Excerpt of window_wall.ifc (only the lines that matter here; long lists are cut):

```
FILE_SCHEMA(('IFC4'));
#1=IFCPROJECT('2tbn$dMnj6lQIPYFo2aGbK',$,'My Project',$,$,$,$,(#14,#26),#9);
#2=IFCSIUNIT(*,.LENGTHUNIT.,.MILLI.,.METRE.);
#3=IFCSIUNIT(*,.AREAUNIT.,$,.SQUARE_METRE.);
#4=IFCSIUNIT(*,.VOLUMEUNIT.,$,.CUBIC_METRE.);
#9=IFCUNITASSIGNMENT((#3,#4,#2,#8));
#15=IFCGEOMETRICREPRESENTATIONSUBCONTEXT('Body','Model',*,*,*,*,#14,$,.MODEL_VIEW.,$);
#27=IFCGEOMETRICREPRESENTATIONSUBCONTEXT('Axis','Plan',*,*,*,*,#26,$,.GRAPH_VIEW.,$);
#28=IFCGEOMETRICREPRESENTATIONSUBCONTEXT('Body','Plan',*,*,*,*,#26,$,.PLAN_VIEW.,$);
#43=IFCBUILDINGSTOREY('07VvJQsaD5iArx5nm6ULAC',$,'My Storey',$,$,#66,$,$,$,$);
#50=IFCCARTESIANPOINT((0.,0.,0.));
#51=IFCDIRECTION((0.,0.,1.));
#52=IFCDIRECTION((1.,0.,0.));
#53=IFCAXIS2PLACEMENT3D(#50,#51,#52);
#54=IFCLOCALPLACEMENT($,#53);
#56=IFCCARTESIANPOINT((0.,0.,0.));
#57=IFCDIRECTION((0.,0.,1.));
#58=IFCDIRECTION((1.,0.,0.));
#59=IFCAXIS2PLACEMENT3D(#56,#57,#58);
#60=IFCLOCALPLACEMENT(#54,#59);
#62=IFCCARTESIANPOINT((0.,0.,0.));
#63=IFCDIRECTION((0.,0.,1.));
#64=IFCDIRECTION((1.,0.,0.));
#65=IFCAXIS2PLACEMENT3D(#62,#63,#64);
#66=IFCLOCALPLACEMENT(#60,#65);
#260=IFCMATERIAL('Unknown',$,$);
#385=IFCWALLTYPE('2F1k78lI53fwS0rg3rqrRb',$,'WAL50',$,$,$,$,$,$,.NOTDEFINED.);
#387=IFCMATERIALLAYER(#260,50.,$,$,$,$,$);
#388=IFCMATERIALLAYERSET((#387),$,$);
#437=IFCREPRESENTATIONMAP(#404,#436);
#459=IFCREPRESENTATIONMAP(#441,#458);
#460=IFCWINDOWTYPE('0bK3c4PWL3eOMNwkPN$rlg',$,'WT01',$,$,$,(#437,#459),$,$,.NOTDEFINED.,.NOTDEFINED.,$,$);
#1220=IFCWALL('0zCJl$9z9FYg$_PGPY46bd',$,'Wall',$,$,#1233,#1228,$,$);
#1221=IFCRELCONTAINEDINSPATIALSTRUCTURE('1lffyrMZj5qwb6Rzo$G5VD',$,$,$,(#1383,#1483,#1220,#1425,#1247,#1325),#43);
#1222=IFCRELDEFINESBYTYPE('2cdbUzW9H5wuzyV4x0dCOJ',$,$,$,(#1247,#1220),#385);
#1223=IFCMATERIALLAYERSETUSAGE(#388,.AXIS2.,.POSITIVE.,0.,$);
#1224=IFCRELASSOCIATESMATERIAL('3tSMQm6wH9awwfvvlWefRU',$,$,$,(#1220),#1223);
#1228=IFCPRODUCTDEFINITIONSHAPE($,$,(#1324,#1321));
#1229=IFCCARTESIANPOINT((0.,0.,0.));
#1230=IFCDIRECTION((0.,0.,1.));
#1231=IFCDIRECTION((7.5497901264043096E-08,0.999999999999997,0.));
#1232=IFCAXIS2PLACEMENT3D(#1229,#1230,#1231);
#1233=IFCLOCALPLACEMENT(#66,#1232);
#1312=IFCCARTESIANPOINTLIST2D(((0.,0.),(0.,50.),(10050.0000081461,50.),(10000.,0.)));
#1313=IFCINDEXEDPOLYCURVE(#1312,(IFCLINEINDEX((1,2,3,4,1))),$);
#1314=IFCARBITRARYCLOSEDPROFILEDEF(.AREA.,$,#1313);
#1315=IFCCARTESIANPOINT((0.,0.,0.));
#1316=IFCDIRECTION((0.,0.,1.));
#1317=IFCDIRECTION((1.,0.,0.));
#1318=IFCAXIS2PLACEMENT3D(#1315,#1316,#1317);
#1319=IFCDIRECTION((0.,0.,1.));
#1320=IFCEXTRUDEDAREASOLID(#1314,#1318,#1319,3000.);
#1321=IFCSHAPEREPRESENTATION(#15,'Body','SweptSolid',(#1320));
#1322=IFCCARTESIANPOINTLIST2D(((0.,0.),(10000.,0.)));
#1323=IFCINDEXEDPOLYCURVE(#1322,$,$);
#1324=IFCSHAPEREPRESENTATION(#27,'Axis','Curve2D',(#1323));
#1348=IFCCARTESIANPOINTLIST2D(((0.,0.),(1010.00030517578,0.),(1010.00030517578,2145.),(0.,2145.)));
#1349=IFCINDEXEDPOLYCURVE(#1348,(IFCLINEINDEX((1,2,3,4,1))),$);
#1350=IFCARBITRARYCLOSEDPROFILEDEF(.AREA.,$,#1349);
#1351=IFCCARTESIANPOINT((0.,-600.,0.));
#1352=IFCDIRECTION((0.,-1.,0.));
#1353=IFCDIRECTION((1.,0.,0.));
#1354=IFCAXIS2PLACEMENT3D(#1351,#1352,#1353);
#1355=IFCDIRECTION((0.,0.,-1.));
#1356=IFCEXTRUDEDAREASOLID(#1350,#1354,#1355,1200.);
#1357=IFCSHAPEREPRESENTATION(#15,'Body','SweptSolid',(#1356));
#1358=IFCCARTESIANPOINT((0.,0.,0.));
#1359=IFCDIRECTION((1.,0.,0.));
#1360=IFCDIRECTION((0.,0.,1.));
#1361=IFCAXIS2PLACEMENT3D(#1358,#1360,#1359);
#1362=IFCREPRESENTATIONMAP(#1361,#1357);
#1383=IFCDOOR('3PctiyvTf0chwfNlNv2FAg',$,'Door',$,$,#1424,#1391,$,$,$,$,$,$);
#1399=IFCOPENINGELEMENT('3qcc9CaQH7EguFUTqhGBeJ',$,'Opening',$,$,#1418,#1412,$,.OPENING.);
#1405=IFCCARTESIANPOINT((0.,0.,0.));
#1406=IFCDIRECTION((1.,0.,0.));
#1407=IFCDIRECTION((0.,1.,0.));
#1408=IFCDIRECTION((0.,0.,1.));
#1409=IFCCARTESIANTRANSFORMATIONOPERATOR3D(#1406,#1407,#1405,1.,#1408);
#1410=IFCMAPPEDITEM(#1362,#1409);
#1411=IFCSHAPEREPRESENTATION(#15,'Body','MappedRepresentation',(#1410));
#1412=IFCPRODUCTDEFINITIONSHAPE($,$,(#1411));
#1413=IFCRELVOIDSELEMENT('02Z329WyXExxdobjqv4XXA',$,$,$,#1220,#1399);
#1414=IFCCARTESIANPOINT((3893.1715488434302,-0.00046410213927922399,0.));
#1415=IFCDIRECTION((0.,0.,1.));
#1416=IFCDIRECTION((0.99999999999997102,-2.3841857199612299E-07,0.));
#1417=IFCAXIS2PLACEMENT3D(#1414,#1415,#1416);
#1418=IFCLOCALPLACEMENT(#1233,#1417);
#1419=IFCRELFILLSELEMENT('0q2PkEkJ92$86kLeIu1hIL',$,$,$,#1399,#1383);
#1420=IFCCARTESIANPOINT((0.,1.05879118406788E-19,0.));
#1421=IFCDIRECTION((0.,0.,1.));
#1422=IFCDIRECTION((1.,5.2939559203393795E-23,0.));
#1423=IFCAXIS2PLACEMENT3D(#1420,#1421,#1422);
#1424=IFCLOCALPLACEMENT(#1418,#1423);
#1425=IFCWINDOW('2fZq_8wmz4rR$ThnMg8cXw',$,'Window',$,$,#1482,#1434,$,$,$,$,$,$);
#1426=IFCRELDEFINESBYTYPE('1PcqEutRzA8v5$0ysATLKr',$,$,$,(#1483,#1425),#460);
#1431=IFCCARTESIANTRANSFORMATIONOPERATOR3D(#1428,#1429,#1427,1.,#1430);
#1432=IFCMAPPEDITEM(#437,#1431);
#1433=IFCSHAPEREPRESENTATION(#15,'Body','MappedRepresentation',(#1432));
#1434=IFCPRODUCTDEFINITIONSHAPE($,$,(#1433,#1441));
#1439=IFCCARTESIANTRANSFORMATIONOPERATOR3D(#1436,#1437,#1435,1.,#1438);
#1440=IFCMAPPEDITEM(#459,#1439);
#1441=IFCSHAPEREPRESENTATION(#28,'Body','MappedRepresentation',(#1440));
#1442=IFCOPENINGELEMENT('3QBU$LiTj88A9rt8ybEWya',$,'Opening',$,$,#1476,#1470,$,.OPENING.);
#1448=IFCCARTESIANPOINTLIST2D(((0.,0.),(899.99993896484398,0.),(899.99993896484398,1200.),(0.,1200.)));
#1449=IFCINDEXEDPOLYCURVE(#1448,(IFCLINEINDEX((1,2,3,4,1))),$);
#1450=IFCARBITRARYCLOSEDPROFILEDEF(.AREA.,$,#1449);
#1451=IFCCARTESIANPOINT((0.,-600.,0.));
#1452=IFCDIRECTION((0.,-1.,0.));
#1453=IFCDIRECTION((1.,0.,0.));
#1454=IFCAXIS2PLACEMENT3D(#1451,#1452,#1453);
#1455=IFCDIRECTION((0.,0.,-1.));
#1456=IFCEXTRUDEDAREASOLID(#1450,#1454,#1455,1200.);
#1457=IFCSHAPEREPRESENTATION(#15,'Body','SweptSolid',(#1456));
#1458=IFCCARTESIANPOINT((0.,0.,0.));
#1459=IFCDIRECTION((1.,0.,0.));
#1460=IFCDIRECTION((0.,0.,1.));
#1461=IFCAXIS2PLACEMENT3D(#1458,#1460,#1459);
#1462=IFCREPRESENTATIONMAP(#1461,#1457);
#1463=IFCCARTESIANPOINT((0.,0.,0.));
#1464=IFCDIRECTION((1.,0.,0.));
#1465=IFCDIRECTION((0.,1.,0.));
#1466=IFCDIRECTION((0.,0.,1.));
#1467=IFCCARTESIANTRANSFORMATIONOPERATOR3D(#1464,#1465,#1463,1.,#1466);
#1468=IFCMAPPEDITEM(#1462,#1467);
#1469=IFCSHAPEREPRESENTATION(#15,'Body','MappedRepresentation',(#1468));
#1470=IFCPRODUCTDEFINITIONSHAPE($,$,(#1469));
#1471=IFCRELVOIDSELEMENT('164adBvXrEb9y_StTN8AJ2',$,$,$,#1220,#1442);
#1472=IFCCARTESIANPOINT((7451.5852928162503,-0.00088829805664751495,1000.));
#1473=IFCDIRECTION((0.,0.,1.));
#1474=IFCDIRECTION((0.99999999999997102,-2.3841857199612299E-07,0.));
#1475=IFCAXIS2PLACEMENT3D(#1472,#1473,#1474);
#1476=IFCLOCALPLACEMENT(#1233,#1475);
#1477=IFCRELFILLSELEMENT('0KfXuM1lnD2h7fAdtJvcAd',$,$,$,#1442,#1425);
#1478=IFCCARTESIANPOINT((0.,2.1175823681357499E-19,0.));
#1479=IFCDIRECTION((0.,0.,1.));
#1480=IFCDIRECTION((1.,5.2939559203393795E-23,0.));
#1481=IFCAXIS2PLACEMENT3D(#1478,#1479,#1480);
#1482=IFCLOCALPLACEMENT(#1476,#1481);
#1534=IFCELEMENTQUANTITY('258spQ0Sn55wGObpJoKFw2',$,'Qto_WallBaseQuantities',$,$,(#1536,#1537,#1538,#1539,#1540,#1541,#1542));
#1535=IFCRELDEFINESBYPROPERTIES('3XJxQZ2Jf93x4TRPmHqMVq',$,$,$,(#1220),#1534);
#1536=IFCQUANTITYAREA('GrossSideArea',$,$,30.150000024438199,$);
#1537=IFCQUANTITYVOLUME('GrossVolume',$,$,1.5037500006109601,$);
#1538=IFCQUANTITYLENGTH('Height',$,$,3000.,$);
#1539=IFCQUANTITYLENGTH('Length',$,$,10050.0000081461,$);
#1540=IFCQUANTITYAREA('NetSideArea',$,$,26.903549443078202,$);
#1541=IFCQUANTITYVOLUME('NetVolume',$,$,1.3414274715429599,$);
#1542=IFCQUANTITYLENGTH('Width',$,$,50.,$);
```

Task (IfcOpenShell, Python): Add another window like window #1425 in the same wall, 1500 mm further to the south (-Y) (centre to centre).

```python
import ifcopenshell
import ifcopenshell.api.feature
import ifcopenshell.api.geometry
import ifcopenshell.api.pset
import ifcopenshell.api.root
import ifcopenshell.geom
import ifcopenshell.util.element
import ifcopenshell.util.placement
import ifcopenshell.util.shape
import ifcopenshell.util.unit

model = ifcopenshell.open("window_wall.ifc")
unit_scale = ifcopenshell.util.unit.calculate_unit_scale(model)
area_scale = ifcopenshell.util.unit.calculate_unit_scale(model, "AREAUNIT")
volume_scale = ifcopenshell.util.unit.calculate_unit_scale(model, "VOLUMEUNIT")
settings = ifcopenshell.geom.settings()


def volume(element):
    """Net volume in cubic metres, openings subtracted."""
    shape = ifcopenshell.geom.create_shape(settings, element)
    return ifcopenshell.util.shape.get_volume(shape.geometry)


window = model.by_guid("2fZq_8wmz4rR$ThnMg8cXw")
opening = window.FillsVoids[0].RelatingOpeningElement
wall = opening.VoidsElements[0].RelatingBuildingElement
before = volume(wall)
shift = ifcopenshell.util.placement.get_local_placement(wall.ObjectPlacement)[:3, 0] * -1.5 / unit_scale

# copy_class copies the void relationship, type, container and properties, but no geometry.
new_opening = ifcopenshell.api.root.copy_class(model, product=opening)
new_opening.Representation = ifcopenshell.util.element.copy_deep(
    model, opening.Representation, exclude=["IfcGeometricRepresentationContext", "IfcRepresentationMap"]
)
new_window = ifcopenshell.api.root.copy_class(model, product=window)
new_window.Representation = ifcopenshell.util.element.copy_deep(
    model, window.Representation, exclude=["IfcGeometricRepresentationContext", "IfcRepresentationMap"]
)
ifcopenshell.api.feature.add_filling(model, opening=new_opening, element=new_window)

for old, new in ((opening, new_opening), (window, new_window)):
    matrix = ifcopenshell.util.placement.get_local_placement(old.ObjectPlacement)
    matrix[:3, 3] += shift
    ifcopenshell.api.geometry.edit_object_placement(model, product=new, matrix=matrix, is_si=False)

after = volume(wall)
thickness = 0.05  # wall thickness in metres

# Update the wall's stored quantities.
qto = model.by_id(ifcopenshell.util.element.get_pset(wall, "Qto_WallBaseQuantities", should_inherit=False)["id"])
ifcopenshell.api.pset.edit_qto(model, qto=qto, properties={
    "NetSideArea": after / thickness / area_scale,
    "NetVolume": after / volume_scale,
})

print(f"wall volume {before:.3f} -> {after:.3f} m3")

model.write("window_wall_edited.ifc")
```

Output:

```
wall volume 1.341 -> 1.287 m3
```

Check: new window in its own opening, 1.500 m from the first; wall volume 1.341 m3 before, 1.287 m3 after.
